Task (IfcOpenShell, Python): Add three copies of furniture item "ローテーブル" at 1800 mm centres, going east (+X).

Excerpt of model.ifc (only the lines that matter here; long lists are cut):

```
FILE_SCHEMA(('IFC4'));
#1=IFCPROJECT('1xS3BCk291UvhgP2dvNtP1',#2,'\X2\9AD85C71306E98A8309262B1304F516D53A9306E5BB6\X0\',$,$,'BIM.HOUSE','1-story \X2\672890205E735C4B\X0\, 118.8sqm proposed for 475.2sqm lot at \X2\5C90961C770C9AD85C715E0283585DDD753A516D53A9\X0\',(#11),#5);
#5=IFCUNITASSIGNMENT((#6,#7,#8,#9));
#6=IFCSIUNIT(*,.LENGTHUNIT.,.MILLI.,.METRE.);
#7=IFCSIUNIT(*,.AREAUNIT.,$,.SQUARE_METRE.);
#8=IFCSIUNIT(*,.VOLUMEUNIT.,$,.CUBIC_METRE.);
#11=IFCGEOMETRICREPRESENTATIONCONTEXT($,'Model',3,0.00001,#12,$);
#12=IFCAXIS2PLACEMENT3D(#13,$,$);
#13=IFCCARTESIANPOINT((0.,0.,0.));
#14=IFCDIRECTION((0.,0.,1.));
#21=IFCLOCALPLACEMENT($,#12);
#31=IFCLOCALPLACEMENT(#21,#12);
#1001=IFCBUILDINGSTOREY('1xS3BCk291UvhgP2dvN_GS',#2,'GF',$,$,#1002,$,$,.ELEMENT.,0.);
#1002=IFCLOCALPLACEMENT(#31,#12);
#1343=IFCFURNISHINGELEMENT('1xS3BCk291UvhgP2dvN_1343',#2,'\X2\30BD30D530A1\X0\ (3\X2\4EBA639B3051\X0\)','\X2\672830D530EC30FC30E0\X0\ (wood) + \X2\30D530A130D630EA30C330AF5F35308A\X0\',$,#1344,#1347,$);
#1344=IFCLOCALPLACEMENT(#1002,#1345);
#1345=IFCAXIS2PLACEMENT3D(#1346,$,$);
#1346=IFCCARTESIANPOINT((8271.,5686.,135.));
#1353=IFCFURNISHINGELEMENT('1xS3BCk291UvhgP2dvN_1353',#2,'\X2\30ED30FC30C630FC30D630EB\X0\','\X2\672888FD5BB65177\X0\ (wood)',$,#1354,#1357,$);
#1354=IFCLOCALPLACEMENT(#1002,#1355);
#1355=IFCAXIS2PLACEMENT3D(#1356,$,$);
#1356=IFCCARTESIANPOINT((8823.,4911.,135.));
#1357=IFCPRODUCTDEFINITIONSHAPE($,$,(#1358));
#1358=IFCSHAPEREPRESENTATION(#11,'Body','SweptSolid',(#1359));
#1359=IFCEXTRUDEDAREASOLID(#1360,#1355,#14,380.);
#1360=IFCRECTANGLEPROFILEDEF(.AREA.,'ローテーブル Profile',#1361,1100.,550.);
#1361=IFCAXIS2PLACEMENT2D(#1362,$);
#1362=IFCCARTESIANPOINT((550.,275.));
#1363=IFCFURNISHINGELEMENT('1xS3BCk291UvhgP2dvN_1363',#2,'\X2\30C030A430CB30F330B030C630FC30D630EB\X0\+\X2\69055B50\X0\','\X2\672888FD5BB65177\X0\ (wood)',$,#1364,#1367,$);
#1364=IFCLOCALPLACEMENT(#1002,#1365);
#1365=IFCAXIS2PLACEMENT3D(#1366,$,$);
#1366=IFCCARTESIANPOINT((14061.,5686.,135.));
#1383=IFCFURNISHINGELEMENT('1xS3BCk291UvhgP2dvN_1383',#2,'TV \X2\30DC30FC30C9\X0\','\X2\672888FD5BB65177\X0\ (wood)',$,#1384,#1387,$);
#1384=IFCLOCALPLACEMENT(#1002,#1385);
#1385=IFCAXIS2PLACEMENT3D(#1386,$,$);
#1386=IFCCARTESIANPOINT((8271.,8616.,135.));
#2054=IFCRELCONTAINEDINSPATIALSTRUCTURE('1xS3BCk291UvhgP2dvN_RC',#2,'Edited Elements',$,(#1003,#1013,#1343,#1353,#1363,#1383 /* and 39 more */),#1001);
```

```python
import numpy as np
import ifcopenshell
import ifcopenshell.api.geometry
import ifcopenshell.api.root
import ifcopenshell.util.element
import ifcopenshell.util.placement
import ifcopenshell.util.unit

model = ifcopenshell.open("model.ifc")
unit_scale = ifcopenshell.util.unit.calculate_unit_scale(model)


def reuse_history(source, copy):
    """copy_class also copies each property set's owner history, people and application; keep the originals."""
    for rel in copy.IsDefinedBy:
        if rel.is_a("IfcRelDefinesByProperties") and (history := rel.RelatingPropertyDefinition.OwnerHistory):
            rel.RelatingPropertyDefinition.OwnerHistory = source.OwnerHistory
            ifcopenshell.util.element.remove_deep2(model, history)


source = model.by_guid("1xS3BCk291UvhgP2dvN_1353")
base = ifcopenshell.util.placement.get_local_placement(source.ObjectPlacement)
step = np.array([1.0, 0.0, 0.0]) * 1.8 / unit_scale

for i in range(1, 4):
    copy = ifcopenshell.api.root.copy_class(model, product=source)
    copy.Representation = ifcopenshell.util.element.copy_deep(
        model, source.Representation, exclude=["IfcGeometricRepresentationContext", "IfcRepresentationMap"]
    )
    reuse_history(source, copy)
    matrix = base.copy()
    matrix[:3, 3] += i * step
    print("added at", matrix[:3, 3].round(3) + 0.0)
    ifcopenshell.api.geometry.edit_object_placement(model, product=copy, matrix=matrix, is_si=False)

model.write("model-out.ifc")
```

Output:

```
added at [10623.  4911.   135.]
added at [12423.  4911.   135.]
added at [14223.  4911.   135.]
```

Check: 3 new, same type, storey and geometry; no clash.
